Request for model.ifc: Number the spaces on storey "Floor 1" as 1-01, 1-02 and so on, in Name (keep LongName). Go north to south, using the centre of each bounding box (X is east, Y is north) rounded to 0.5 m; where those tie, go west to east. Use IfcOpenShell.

First a look at what the model holds.

```python
import ifcopenshell
import ifcopenshell.util.element
import ifcopenshell.util.placement

model = ifcopenshell.open("model.ifc")
print(model.schema)
storey = next(s for s in model.by_type("IfcBuildingStorey") if s.Name == "Floor 1")
spaces = [e for e in ifcopenshell.util.element.get_decomposition(storey) if e.is_a("IfcSpace")]
for e in sorted(spaces, key=lambda e: e.id()):
    origin = ifcopenshell.util.placement.get_local_placement(e.ObjectPlacement)[:3, 3]
    print(e.id(), e.Name, e.LongName, origin.round(2) + 0.0, sep=" | ")
```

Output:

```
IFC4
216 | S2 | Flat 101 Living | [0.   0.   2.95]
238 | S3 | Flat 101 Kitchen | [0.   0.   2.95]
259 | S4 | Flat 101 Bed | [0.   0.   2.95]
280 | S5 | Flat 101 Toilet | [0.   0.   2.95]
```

```python
import ifcopenshell
import ifcopenshell.geom
import ifcopenshell.util.element
import ifcopenshell.util.shape

model = ifcopenshell.open("model.ifc")
settings = ifcopenshell.geom.settings()
settings.set("use-world-coords", True)


def centre(element):
    shape = ifcopenshell.geom.create_shape(settings, element)
    return ifcopenshell.util.shape.get_bbox_centroid(shape.geometry)


storey = next(s for s in model.by_type("IfcBuildingStorey") if s.Name == "Floor 1")
spaces = [e for e in ifcopenshell.util.element.get_decomposition(storey) if e.is_a("IfcSpace")]

# Insertion points can sit at a corner or the storey origin, so sort by the geometry (in metres).
centres = {e: centre(e) for e in spaces}
spaces.sort(key=lambda e: (-round(centres[e][1] / 0.5), centres[e][0]))

for i, e in enumerate(spaces, start=1):
    number = f"1-{i:02d}"
    e.Name = number
    print(e.id(), number)

model.write("model_edited.ifc")
```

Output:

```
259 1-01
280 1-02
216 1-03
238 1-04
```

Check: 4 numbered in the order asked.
